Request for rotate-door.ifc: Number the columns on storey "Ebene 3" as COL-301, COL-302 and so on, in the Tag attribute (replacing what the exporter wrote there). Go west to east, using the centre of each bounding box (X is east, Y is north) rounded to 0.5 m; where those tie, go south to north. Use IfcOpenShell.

First a look at what the model holds.

```python
import ifcopenshell
import ifcopenshell.util.element
import ifcopenshell.util.placement

model = ifcopenshell.open("rotate-door.ifc")
print(model.schema)
storey = next(s for s in model.by_type("IfcBuildingStorey") if s.Name == "Ebene 3")
columns = [e for e in ifcopenshell.util.element.get_decomposition(storey) if e.is_a("IfcColumn")]
for e in sorted(columns, key=lambda e: e.id()):
    origin = ifcopenshell.util.placement.get_local_placement(e.ObjectPlacement)[:3, 3]
    print(e.id(), e.Tag, e.Name, origin.round(2) + 0.0, sep=" | ")
```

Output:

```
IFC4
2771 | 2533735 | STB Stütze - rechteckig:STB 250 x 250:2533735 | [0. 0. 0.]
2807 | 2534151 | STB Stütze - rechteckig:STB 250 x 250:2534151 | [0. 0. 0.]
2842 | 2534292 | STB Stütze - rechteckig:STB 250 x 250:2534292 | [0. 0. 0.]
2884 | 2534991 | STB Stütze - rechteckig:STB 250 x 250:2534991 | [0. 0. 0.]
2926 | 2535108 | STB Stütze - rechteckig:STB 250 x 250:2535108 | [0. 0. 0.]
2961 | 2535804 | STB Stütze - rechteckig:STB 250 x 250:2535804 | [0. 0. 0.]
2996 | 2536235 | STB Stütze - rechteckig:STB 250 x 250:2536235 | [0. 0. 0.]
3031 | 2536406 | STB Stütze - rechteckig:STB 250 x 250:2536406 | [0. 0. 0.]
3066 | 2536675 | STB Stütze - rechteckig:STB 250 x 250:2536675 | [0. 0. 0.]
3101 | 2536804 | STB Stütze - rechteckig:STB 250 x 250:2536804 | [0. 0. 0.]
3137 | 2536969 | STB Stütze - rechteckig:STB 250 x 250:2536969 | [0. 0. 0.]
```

```python
import ifcopenshell
import ifcopenshell.geom
import ifcopenshell.util.element
import ifcopenshell.util.shape

model = ifcopenshell.open("rotate-door.ifc")
settings = ifcopenshell.geom.settings()
settings.set("use-world-coords", True)


def centre(element):
    shape = ifcopenshell.geom.create_shape(settings, element)
    return ifcopenshell.util.shape.get_bbox_centroid(shape.geometry)


storey = next(s for s in model.by_type("IfcBuildingStorey") if s.Name == "Ebene 3")
columns = [e for e in ifcopenshell.util.element.get_decomposition(storey) if e.is_a("IfcColumn")]

# Insertion points can sit at a corner or the storey origin, so sort by the geometry (in metres).
centres = {e: centre(e) for e in columns}
columns.sort(key=lambda e: (round(centres[e][0] / 0.5), centres[e][1]))

for i, e in enumerate(columns, start=1):
    number = f"COL-3{i:02d}"
    e.Tag = number
    print(e.id(), number)

model.write("rotate-door-out.ifc")
```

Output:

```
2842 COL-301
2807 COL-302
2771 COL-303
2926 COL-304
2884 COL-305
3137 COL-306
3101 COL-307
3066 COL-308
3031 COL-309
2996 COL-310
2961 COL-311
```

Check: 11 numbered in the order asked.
